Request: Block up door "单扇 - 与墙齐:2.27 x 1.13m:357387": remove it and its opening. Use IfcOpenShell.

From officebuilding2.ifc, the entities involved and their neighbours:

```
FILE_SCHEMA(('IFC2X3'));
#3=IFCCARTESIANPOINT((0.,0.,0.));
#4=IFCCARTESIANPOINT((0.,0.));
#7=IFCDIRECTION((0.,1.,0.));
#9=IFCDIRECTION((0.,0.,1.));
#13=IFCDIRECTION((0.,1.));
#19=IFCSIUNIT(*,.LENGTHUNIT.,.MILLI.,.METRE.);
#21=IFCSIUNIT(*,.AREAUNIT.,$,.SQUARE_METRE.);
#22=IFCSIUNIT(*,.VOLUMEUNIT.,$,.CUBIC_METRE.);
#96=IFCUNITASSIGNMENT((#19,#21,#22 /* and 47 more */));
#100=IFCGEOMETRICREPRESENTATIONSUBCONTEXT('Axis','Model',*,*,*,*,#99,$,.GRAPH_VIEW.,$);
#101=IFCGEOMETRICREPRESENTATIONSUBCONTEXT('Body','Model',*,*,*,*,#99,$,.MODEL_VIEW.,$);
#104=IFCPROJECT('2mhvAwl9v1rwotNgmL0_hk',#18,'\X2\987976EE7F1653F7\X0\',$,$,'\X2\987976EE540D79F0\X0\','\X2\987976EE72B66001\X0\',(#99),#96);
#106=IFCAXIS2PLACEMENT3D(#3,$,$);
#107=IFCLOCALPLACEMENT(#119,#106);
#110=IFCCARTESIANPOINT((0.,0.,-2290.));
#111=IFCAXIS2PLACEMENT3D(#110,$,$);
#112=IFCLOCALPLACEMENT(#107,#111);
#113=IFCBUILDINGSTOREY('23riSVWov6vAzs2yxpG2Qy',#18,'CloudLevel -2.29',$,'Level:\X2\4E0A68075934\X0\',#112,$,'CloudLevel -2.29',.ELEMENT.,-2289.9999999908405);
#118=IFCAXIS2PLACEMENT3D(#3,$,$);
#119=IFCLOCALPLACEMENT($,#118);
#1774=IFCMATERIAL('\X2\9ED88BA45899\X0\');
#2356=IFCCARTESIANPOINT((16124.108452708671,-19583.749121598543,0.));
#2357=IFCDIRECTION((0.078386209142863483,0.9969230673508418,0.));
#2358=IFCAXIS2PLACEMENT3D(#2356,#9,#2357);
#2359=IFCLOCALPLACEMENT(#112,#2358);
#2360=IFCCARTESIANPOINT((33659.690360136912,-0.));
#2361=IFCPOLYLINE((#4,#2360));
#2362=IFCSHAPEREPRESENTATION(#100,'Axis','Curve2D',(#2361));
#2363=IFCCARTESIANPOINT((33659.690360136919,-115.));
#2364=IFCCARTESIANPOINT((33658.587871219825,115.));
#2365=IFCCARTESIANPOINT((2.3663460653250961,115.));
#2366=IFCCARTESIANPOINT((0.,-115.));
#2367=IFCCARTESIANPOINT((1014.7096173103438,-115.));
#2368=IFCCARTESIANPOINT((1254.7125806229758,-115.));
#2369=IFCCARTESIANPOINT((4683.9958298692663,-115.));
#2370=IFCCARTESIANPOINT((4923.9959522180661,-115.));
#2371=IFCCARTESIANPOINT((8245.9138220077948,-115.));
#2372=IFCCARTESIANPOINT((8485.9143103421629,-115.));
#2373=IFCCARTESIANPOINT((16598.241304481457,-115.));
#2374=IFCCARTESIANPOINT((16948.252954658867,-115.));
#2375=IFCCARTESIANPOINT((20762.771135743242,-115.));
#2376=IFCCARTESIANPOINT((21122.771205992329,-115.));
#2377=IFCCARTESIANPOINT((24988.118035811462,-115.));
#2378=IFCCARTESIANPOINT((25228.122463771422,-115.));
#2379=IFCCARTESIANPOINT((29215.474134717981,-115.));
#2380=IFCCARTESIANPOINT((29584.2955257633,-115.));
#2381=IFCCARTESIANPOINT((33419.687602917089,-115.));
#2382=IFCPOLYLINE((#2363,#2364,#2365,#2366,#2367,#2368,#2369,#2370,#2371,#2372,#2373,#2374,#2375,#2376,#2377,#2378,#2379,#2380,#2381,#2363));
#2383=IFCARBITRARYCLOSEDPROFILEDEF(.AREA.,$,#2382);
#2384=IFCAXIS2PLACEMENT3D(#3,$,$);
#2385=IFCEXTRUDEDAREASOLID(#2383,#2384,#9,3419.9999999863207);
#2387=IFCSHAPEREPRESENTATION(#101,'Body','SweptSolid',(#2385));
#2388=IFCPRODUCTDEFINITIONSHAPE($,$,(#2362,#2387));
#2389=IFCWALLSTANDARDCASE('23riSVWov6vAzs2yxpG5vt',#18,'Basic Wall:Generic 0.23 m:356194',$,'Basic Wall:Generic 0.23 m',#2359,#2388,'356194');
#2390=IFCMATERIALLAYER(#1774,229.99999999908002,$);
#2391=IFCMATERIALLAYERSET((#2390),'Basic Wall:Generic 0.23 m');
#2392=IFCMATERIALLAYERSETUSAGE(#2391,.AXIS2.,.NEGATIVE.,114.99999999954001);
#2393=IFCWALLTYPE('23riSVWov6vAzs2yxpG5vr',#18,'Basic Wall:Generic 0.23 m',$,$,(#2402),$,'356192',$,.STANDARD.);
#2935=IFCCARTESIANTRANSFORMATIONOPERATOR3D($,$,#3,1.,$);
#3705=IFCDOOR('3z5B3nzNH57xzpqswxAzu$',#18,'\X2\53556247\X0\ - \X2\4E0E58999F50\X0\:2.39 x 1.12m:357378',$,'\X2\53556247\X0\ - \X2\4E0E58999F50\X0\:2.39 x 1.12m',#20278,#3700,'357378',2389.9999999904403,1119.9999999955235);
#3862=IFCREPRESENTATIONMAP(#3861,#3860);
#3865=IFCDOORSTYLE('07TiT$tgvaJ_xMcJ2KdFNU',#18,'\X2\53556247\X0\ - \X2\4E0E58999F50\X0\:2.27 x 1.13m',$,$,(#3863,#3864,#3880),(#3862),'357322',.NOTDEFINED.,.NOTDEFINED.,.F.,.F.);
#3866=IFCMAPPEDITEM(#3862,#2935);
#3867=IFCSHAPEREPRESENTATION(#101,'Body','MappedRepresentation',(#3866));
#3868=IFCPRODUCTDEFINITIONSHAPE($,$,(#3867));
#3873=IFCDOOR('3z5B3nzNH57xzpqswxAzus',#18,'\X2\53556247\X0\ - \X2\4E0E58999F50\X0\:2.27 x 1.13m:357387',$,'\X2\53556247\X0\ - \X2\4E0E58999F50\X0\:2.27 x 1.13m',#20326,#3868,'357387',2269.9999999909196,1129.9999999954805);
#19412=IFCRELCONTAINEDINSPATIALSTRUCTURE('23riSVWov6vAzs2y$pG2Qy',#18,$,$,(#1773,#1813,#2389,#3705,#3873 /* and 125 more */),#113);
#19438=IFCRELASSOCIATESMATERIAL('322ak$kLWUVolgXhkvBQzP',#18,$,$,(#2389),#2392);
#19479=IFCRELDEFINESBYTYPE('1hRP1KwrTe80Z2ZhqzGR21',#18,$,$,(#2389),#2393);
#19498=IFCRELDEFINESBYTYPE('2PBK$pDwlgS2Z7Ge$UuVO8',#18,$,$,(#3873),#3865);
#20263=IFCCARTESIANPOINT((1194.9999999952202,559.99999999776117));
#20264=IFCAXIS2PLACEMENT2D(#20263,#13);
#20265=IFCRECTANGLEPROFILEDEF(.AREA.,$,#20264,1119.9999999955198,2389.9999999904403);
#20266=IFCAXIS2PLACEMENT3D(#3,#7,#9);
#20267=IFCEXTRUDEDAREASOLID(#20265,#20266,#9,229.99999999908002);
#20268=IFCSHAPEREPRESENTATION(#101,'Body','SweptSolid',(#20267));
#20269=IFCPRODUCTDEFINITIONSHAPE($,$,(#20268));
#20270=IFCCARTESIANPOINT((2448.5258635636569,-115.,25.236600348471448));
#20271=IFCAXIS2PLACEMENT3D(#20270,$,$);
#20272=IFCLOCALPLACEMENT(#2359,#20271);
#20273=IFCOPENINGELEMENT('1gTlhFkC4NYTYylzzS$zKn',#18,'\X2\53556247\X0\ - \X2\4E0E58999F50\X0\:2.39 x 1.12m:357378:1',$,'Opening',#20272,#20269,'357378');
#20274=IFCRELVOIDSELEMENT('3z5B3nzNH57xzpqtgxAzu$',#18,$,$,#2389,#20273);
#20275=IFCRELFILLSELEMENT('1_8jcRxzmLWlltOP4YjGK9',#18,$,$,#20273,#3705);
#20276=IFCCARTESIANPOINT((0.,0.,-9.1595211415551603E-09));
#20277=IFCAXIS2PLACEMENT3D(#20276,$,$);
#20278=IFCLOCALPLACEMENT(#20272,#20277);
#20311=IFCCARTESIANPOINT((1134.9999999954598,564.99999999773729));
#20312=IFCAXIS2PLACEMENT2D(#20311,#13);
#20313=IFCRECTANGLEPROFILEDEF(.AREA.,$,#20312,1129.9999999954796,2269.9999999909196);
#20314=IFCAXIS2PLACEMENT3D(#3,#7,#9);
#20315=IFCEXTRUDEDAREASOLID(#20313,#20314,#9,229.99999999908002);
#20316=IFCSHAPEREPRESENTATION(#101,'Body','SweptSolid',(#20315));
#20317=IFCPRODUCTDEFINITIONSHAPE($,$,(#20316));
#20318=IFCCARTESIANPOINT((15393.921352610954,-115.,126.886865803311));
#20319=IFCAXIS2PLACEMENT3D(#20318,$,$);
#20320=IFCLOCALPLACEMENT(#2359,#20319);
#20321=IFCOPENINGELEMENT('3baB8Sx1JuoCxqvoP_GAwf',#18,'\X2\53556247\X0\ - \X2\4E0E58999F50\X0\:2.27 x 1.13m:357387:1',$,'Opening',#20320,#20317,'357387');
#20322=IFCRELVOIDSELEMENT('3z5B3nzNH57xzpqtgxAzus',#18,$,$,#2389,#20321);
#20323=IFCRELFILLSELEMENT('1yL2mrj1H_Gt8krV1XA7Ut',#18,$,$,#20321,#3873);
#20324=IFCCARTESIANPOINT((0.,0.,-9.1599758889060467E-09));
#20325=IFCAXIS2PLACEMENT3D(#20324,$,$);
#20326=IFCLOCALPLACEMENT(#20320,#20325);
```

```python
import ifcopenshell
import ifcopenshell.api.feature
import ifcopenshell.api.root
import ifcopenshell.geom
import ifcopenshell.util.shape

model = ifcopenshell.open("officebuilding2.ifc")
settings = ifcopenshell.geom.settings()


def volume(element):
    """Net volume in cubic metres, openings subtracted."""
    shape = ifcopenshell.geom.create_shape(settings, element)
    return ifcopenshell.util.shape.get_volume(shape.geometry)


door = model.by_guid("3z5B3nzNH57xzpqswxAzus")
opening = door.FillsVoids[0].RelatingOpeningElement
wall = opening.VoidsElements[0].RelatingBuildingElement
before = volume(wall)

ifcopenshell.api.root.remove_product(model, product=door)
ifcopenshell.api.feature.remove_feature(model, feature=opening)

after = volume(wall)

print(f"wall volume {before:.3f} -> {after:.3f} m3")

model.write("officebuilding2_updated.ifc")
```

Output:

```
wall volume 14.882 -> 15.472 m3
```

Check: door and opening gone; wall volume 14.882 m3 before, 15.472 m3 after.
